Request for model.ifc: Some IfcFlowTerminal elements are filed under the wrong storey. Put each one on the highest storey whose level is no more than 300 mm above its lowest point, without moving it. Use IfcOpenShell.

First a look at what the model holds.

```python
import ifcopenshell
import ifcopenshell.util.element
import ifcopenshell.util.placement

model = ifcopenshell.open("model.ifc")
print(model.schema)
for storey in model.by_type("IfcBuildingStorey"):
    level = ifcopenshell.util.placement.get_storey_elevation(storey)
    count = sum(e.is_a("IfcFlowTerminal") for e in ifcopenshell.util.element.get_contained(storey))
    print(storey.id(), storey.Name, round(level, 3), count, sep=" | ")
```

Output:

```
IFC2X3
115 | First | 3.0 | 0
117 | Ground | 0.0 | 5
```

```python
import ifcopenshell
import ifcopenshell.api.spatial
import ifcopenshell.geom
import ifcopenshell.util.element
import ifcopenshell.util.placement
import ifcopenshell.util.shape
import ifcopenshell.util.unit

model = ifcopenshell.open("model.ifc")
unit_scale = ifcopenshell.util.unit.calculate_unit_scale(model)
settings = ifcopenshell.geom.settings()

levels = sorted(
    ((ifcopenshell.util.placement.get_storey_elevation(s) * unit_scale, s) for s in model.by_type("IfcBuildingStorey")),
    key=lambda pair: pair[0],
)

for e in model.by_type("IfcFlowTerminal"):
    current = e.ContainedInStructure[0].RelatingStructure if e.ContainedInStructure else None
    if current is None or not current.is_a("IfcBuildingStorey"):
        continue
    shape = ifcopenshell.geom.create_shape(settings, e)
    bottom = ifcopenshell.util.shape.get_shape_bottom_elevation(shape, shape.geometry)
    below = [s for level, s in levels if level <= bottom + 0.3]
    storey = below[-1] if below else levels[0][1]
    if storey != current:
        # assign_container keeps the world position.
        ifcopenshell.api.spatial.assign_container(model, products=[e], relating_structure=storey)
        print(e.id(), current.Name, "->", storey.Name)

model.write("model_v2.ifc")
```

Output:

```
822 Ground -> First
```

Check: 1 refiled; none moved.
